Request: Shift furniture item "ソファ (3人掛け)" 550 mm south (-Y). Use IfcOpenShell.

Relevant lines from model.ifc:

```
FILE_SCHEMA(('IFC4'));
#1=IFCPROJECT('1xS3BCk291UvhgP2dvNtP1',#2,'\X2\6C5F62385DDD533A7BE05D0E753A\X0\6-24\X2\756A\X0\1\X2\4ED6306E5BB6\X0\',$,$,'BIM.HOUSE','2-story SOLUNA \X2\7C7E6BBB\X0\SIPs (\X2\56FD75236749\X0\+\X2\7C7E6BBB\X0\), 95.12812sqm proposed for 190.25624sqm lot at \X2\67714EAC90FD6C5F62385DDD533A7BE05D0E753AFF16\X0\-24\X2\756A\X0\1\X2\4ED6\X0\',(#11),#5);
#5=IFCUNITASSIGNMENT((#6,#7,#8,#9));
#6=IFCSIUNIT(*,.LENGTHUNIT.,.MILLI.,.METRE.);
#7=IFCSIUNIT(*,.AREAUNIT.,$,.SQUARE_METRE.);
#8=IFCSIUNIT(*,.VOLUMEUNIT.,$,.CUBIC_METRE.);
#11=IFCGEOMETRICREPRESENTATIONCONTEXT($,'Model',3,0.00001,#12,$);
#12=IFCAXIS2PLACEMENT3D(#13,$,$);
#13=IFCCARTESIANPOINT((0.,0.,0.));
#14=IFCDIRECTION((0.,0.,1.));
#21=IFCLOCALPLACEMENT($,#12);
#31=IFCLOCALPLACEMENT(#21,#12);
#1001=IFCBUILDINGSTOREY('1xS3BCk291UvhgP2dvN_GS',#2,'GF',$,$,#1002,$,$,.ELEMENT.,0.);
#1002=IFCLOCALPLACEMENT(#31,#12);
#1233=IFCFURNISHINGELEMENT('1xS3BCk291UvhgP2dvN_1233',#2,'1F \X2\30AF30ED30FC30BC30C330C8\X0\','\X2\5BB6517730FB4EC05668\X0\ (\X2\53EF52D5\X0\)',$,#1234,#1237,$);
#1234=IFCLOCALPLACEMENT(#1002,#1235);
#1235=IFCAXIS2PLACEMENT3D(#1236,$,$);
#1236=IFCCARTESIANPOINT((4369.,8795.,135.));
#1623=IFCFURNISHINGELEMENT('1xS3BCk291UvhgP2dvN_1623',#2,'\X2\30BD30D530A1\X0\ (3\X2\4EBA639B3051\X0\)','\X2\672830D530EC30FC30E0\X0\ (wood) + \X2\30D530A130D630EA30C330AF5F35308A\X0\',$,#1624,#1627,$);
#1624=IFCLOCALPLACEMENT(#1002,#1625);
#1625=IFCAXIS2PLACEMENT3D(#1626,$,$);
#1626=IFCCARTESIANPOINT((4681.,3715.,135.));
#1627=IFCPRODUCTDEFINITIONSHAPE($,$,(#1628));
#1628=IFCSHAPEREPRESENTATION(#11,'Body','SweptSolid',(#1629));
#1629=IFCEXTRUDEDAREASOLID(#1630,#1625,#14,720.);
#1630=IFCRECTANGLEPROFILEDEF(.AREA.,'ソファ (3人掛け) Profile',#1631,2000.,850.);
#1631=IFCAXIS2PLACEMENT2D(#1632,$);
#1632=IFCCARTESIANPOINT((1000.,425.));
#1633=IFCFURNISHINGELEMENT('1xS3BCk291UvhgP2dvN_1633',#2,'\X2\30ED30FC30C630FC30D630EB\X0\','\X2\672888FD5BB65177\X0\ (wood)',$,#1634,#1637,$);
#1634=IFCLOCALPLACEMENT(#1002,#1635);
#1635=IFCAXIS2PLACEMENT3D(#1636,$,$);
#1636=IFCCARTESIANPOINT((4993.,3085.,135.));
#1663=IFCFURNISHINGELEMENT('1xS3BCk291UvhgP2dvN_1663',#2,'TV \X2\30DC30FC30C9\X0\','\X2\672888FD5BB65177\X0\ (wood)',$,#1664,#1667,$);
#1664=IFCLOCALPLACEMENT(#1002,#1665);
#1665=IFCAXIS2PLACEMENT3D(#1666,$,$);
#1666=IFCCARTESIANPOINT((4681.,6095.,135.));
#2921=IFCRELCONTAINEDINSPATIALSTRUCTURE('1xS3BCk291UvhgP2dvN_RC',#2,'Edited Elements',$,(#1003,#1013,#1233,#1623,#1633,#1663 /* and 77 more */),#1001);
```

```python
import ifcopenshell
import ifcopenshell.api.geometry
import ifcopenshell.util.placement
import ifcopenshell.util.unit

model = ifcopenshell.open("model.ifc")
unit_scale = ifcopenshell.util.unit.calculate_unit_scale(model)

item = model.by_id(1623)
matrix = ifcopenshell.util.placement.get_local_placement(item.ObjectPlacement)
matrix[1, 3] -= 0.55 / unit_scale
ifcopenshell.api.geometry.edit_object_placement(model, product=item, matrix=matrix, is_si=False)

print(ifcopenshell.util.placement.get_local_placement(item.ObjectPlacement).round(3) + 0.0)

model.write("model_rev.ifc")
```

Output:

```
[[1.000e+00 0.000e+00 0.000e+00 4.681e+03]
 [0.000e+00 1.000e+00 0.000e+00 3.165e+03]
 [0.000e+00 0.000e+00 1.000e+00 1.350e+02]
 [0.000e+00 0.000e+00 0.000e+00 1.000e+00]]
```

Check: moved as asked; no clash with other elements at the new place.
